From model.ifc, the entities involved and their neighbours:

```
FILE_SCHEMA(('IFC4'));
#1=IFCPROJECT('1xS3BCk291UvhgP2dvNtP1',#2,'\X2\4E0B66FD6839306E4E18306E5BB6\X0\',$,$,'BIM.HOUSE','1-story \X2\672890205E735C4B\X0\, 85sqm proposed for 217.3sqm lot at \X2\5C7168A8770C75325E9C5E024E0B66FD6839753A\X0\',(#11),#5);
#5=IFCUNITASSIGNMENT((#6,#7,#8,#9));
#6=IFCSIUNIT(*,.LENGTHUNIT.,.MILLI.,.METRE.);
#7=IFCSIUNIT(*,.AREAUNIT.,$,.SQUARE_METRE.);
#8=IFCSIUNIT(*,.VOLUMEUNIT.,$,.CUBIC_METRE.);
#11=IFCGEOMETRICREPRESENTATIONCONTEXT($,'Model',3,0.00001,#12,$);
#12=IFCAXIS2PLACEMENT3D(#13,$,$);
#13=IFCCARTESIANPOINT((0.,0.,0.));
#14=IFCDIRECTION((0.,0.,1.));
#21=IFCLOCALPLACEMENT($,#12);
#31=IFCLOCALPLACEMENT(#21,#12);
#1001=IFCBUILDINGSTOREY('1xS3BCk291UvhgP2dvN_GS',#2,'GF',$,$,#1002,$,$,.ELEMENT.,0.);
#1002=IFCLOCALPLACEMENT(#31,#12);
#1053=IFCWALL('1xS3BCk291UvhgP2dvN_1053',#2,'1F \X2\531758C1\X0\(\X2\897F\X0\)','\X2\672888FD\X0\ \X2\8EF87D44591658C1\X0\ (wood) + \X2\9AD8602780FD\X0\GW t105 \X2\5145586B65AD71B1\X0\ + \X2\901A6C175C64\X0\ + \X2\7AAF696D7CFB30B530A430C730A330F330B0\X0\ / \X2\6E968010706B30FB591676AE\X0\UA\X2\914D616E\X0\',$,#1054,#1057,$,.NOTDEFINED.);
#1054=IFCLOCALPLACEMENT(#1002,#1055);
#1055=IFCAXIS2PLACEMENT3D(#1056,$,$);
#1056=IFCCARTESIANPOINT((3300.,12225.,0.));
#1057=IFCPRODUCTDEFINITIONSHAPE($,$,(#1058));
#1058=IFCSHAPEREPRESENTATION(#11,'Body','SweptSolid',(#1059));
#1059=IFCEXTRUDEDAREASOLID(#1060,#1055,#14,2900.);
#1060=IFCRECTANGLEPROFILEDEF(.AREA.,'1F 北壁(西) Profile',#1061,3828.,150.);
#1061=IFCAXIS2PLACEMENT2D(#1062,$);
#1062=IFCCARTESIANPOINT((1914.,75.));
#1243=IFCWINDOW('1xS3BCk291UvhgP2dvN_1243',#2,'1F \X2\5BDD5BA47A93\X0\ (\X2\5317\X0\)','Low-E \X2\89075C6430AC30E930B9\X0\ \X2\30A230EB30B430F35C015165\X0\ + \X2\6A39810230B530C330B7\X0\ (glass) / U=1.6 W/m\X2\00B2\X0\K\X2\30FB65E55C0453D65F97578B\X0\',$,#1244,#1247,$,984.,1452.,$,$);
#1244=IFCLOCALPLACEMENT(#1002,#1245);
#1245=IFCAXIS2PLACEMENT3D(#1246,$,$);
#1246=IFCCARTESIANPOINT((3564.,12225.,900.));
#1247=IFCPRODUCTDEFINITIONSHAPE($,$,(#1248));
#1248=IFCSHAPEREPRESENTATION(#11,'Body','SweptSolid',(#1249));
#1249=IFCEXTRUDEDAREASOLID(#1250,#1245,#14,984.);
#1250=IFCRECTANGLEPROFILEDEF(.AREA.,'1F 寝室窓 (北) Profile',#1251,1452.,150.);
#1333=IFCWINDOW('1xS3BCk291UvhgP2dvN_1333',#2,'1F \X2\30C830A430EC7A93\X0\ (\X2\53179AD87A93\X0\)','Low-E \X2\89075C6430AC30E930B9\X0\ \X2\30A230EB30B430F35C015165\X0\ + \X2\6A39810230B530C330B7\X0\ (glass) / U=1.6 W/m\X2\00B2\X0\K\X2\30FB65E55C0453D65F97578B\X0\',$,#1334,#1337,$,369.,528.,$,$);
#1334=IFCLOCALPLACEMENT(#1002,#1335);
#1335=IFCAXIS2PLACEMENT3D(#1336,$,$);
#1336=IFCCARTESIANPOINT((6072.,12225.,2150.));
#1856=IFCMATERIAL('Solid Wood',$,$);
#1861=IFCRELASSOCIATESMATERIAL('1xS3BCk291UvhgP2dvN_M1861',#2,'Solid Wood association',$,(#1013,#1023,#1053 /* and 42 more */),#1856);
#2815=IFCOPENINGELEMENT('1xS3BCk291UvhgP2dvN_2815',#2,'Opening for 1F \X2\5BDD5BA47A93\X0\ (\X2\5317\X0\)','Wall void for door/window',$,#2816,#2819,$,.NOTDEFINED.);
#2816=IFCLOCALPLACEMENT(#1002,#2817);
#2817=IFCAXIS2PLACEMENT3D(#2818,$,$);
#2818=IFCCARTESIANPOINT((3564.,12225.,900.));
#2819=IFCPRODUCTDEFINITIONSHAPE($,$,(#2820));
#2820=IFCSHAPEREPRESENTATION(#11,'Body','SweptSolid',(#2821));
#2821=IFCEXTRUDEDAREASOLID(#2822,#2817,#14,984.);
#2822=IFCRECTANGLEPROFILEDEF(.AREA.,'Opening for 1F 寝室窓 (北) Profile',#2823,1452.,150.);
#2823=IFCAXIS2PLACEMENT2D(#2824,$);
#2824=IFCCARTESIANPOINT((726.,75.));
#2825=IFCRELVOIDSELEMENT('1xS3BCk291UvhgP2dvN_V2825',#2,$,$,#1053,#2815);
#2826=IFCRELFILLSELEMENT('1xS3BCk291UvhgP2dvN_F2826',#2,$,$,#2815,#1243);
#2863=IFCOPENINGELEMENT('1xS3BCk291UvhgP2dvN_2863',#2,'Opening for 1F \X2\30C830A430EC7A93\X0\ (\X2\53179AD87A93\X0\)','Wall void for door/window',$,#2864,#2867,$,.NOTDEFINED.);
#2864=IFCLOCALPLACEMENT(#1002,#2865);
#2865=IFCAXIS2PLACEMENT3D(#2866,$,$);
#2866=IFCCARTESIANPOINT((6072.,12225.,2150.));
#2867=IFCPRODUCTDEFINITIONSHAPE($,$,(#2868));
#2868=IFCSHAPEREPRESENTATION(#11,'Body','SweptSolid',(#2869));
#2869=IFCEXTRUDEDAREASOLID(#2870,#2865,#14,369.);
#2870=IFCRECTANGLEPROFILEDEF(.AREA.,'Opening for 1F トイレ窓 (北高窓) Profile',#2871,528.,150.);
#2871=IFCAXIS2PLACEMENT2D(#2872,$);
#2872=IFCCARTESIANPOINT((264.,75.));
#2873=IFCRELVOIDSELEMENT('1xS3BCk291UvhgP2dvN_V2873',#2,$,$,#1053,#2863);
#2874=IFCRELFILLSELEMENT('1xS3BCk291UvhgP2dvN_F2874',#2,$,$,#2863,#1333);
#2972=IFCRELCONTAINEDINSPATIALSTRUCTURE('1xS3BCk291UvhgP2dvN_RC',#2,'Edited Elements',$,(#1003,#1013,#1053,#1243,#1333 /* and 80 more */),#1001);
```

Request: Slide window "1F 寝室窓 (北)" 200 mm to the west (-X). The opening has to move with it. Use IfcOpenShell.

```python
import ifcopenshell
import ifcopenshell.api.geometry
import ifcopenshell.util.placement
import ifcopenshell.util.unit

model = ifcopenshell.open("model.ifc")
unit_scale = ifcopenshell.util.unit.calculate_unit_scale(model)

window = model.by_guid("1xS3BCk291UvhgP2dvN_1243")
opening = window.FillsVoids[0].RelatingOpeningElement
wall = opening.VoidsElements[0].RelatingBuildingElement

wall_matrix = ifcopenshell.util.placement.get_local_placement(wall.ObjectPlacement)
shift = wall_matrix[:3, 0] * -0.2 / unit_scale
before = ifcopenshell.util.placement.get_local_placement(window.ObjectPlacement)[:3, 3].copy()

# The window is not placed relative to its opening, so move both.
for product in (opening, window):
    matrix = ifcopenshell.util.placement.get_local_placement(product.ObjectPlacement)
    matrix[:3, 3] += shift
    ifcopenshell.api.geometry.edit_object_placement(model, product=product, matrix=matrix, is_si=False)

after = ifcopenshell.util.placement.get_local_placement(window.ObjectPlacement)[:3, 3]
print("window moved by", (after - before).round(3) + 0.0)

model.write("model_edited.ifc")
```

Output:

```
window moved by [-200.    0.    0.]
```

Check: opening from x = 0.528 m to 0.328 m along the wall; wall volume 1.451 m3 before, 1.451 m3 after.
